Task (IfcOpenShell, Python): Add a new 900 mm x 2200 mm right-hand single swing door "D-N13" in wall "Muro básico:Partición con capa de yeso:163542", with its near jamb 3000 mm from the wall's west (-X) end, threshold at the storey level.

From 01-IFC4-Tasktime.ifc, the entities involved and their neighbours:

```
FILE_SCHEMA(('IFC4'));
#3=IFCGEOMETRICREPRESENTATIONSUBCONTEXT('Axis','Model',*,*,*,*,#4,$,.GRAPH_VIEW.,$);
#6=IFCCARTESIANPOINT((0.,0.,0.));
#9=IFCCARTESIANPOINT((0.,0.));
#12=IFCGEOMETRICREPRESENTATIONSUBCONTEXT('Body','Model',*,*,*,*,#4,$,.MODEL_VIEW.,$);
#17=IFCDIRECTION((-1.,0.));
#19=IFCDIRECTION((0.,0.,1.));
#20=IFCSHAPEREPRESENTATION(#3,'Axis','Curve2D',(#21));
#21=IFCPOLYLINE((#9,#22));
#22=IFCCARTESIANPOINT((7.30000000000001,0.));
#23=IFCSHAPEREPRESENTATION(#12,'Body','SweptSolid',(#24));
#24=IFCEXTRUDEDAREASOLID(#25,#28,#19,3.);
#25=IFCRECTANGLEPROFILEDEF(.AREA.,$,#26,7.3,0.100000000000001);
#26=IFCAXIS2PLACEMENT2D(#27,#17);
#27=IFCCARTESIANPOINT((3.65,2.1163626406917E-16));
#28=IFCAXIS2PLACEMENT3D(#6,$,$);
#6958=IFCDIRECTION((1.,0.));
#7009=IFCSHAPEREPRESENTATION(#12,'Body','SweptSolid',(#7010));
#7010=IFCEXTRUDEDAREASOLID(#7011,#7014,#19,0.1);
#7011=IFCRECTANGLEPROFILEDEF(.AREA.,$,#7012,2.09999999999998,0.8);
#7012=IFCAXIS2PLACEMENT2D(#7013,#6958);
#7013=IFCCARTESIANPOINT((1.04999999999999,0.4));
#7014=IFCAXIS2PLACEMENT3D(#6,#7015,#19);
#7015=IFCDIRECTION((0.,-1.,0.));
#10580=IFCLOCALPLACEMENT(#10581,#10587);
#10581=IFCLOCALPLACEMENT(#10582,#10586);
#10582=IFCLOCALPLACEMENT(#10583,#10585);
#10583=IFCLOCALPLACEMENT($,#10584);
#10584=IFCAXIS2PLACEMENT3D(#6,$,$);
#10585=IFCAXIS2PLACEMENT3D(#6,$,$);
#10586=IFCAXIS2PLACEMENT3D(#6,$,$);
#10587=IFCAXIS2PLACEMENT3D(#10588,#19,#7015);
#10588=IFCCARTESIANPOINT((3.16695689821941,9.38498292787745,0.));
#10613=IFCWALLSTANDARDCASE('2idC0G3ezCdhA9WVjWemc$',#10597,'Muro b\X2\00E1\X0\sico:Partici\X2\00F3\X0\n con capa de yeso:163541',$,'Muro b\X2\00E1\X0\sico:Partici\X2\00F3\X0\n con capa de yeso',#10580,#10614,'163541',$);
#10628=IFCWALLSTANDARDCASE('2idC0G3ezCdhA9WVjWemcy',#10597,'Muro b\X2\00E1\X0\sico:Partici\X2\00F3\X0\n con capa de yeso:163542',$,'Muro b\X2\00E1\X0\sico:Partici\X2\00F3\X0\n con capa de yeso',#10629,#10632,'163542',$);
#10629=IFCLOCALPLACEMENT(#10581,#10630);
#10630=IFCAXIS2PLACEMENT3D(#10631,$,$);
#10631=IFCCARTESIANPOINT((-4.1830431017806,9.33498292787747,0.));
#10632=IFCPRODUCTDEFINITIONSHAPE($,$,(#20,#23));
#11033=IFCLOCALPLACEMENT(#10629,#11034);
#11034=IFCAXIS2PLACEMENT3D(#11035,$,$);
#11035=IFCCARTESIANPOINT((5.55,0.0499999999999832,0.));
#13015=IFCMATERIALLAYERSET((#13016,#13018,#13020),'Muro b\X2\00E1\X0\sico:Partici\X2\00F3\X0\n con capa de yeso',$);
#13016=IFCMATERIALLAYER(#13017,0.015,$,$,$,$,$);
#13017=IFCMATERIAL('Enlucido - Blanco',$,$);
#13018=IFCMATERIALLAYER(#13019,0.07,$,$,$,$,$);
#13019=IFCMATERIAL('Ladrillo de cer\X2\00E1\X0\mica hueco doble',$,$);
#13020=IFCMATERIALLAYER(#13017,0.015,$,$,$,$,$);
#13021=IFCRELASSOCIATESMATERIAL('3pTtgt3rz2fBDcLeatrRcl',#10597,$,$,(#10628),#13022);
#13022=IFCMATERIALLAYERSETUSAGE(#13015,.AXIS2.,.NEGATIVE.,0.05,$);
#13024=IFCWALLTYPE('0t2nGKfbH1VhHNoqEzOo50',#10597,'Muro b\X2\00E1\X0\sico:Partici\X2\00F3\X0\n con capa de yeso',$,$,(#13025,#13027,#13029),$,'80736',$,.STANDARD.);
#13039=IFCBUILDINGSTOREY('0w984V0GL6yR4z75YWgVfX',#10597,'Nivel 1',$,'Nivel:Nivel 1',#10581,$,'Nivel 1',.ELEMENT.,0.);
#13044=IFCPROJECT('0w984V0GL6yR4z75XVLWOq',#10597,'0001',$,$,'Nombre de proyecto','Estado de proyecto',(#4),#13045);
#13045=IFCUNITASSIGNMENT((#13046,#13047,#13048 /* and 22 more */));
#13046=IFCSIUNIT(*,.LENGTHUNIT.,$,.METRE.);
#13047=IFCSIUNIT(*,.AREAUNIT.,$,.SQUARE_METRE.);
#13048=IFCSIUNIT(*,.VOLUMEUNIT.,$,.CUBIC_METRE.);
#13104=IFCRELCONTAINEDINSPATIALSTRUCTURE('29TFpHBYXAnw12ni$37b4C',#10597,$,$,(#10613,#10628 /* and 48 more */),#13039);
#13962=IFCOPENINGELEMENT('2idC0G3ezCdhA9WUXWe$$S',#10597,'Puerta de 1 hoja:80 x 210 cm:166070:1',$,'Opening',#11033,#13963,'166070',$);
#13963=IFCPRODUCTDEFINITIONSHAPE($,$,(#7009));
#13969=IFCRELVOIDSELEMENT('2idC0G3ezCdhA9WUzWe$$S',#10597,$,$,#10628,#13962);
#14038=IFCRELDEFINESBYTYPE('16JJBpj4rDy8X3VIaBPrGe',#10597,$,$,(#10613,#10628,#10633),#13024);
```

```python
import numpy as np
import ifcopenshell
import ifcopenshell.api.feature
import ifcopenshell.api.geometry
import ifcopenshell.api.root
import ifcopenshell.api.spatial
import ifcopenshell.geom
import ifcopenshell.util.element
import ifcopenshell.util.placement
import ifcopenshell.util.representation
import ifcopenshell.util.shape
import ifcopenshell.util.unit

model = ifcopenshell.open("01-IFC4-Tasktime.ifc")
unit_scale = ifcopenshell.util.unit.calculate_unit_scale(model)
settings = ifcopenshell.geom.settings()


def volume(element):
    """Net volume in cubic metres, openings subtracted."""
    shape = ifcopenshell.geom.create_shape(settings, element)
    return ifcopenshell.util.shape.get_volume(shape.geometry)


wall = model.by_guid("2idC0G3ezCdhA9WVjWemcy")
storey = ifcopenshell.util.element.get_container(wall, ifc_class="IfcBuildingStorey")
context = ifcopenshell.util.representation.get_context(model, "Model", "Body", "MODEL_VIEW")
before = volume(wall)

width, height, from_end, sill = 0.9, 2.2, 3, 0.0  # metres

# The wall runs along its own X axis, and the end named is its -X end.
wall_shape = ifcopenshell.geom.create_shape(settings, wall)
x, y, z = ifcopenshell.util.shape.get_vertices(wall_shape.geometry).T
start = x.min() + from_end
face, thickness = float(y.min()), float(y.max() - y.min())
wall_matrix = ifcopenshell.util.placement.get_local_placement(wall.ObjectPlacement)
level = ifcopenshell.util.placement.get_local_placement(storey.ObjectPlacement)[2, 3]


def in_wall(x, y):
    """Placement at x, y metres in the wall's axes, at sill height."""
    matrix = wall_matrix.copy()
    matrix[:, 3] = wall_matrix @ np.array([x / unit_scale, y / unit_scale, 0.0, 1.0])
    matrix[2, 3] = level + sill / unit_scale
    return matrix


# Opening: a box that overshoots both wall faces by 50 mm.
opening = ifcopenshell.api.root.create_entity(model, ifc_class="IfcOpeningElement", predefined_type="OPENING")
box = ifcopenshell.api.geometry.add_wall_representation(
    model, context=context, length=width, height=height, thickness=thickness + 0.1
)
ifcopenshell.api.geometry.assign_representation(model, product=opening, representation=box)
ifcopenshell.api.geometry.edit_object_placement(model, product=opening, matrix=in_wall(start, face - 0.05), is_si=False)
ifcopenshell.api.feature.add_feature(model, feature=opening, element=wall)

door = ifcopenshell.api.root.create_entity(model, ifc_class="IfcDoor", name="D-N13", predefined_type="DOOR")
door.OverallWidth, door.OverallHeight = width / unit_scale, height / unit_scale
door.OperationType = "SINGLE_SWING_RIGHT"
body = ifcopenshell.api.geometry.add_door_representation(
    model,
    context=context,
    overall_width=door.OverallWidth,
    overall_height=door.OverallHeight,
    operation_type="SINGLE_SWING_RIGHT",
    lining_properties={"LiningDepth": thickness / unit_scale, "ThresholdDepth": thickness / unit_scale},
)
ifcopenshell.api.geometry.assign_representation(model, product=door, representation=body)
ifcopenshell.api.spatial.assign_container(model, products=[door], relating_structure=storey)
ifcopenshell.api.feature.add_filling(model, opening=opening, element=door)

# The lining spans the wall, so the door starts at the wall face.
ifcopenshell.api.geometry.edit_object_placement(model, product=door, matrix=in_wall(start, face), is_si=False)

after = volume(wall)

print(f"wall volume {before:.3f} -> {after:.3f} m3")

model.write("01-IFC4-Tasktime_rev.ifc")
```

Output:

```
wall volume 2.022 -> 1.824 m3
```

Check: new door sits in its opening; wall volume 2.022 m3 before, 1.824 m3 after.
